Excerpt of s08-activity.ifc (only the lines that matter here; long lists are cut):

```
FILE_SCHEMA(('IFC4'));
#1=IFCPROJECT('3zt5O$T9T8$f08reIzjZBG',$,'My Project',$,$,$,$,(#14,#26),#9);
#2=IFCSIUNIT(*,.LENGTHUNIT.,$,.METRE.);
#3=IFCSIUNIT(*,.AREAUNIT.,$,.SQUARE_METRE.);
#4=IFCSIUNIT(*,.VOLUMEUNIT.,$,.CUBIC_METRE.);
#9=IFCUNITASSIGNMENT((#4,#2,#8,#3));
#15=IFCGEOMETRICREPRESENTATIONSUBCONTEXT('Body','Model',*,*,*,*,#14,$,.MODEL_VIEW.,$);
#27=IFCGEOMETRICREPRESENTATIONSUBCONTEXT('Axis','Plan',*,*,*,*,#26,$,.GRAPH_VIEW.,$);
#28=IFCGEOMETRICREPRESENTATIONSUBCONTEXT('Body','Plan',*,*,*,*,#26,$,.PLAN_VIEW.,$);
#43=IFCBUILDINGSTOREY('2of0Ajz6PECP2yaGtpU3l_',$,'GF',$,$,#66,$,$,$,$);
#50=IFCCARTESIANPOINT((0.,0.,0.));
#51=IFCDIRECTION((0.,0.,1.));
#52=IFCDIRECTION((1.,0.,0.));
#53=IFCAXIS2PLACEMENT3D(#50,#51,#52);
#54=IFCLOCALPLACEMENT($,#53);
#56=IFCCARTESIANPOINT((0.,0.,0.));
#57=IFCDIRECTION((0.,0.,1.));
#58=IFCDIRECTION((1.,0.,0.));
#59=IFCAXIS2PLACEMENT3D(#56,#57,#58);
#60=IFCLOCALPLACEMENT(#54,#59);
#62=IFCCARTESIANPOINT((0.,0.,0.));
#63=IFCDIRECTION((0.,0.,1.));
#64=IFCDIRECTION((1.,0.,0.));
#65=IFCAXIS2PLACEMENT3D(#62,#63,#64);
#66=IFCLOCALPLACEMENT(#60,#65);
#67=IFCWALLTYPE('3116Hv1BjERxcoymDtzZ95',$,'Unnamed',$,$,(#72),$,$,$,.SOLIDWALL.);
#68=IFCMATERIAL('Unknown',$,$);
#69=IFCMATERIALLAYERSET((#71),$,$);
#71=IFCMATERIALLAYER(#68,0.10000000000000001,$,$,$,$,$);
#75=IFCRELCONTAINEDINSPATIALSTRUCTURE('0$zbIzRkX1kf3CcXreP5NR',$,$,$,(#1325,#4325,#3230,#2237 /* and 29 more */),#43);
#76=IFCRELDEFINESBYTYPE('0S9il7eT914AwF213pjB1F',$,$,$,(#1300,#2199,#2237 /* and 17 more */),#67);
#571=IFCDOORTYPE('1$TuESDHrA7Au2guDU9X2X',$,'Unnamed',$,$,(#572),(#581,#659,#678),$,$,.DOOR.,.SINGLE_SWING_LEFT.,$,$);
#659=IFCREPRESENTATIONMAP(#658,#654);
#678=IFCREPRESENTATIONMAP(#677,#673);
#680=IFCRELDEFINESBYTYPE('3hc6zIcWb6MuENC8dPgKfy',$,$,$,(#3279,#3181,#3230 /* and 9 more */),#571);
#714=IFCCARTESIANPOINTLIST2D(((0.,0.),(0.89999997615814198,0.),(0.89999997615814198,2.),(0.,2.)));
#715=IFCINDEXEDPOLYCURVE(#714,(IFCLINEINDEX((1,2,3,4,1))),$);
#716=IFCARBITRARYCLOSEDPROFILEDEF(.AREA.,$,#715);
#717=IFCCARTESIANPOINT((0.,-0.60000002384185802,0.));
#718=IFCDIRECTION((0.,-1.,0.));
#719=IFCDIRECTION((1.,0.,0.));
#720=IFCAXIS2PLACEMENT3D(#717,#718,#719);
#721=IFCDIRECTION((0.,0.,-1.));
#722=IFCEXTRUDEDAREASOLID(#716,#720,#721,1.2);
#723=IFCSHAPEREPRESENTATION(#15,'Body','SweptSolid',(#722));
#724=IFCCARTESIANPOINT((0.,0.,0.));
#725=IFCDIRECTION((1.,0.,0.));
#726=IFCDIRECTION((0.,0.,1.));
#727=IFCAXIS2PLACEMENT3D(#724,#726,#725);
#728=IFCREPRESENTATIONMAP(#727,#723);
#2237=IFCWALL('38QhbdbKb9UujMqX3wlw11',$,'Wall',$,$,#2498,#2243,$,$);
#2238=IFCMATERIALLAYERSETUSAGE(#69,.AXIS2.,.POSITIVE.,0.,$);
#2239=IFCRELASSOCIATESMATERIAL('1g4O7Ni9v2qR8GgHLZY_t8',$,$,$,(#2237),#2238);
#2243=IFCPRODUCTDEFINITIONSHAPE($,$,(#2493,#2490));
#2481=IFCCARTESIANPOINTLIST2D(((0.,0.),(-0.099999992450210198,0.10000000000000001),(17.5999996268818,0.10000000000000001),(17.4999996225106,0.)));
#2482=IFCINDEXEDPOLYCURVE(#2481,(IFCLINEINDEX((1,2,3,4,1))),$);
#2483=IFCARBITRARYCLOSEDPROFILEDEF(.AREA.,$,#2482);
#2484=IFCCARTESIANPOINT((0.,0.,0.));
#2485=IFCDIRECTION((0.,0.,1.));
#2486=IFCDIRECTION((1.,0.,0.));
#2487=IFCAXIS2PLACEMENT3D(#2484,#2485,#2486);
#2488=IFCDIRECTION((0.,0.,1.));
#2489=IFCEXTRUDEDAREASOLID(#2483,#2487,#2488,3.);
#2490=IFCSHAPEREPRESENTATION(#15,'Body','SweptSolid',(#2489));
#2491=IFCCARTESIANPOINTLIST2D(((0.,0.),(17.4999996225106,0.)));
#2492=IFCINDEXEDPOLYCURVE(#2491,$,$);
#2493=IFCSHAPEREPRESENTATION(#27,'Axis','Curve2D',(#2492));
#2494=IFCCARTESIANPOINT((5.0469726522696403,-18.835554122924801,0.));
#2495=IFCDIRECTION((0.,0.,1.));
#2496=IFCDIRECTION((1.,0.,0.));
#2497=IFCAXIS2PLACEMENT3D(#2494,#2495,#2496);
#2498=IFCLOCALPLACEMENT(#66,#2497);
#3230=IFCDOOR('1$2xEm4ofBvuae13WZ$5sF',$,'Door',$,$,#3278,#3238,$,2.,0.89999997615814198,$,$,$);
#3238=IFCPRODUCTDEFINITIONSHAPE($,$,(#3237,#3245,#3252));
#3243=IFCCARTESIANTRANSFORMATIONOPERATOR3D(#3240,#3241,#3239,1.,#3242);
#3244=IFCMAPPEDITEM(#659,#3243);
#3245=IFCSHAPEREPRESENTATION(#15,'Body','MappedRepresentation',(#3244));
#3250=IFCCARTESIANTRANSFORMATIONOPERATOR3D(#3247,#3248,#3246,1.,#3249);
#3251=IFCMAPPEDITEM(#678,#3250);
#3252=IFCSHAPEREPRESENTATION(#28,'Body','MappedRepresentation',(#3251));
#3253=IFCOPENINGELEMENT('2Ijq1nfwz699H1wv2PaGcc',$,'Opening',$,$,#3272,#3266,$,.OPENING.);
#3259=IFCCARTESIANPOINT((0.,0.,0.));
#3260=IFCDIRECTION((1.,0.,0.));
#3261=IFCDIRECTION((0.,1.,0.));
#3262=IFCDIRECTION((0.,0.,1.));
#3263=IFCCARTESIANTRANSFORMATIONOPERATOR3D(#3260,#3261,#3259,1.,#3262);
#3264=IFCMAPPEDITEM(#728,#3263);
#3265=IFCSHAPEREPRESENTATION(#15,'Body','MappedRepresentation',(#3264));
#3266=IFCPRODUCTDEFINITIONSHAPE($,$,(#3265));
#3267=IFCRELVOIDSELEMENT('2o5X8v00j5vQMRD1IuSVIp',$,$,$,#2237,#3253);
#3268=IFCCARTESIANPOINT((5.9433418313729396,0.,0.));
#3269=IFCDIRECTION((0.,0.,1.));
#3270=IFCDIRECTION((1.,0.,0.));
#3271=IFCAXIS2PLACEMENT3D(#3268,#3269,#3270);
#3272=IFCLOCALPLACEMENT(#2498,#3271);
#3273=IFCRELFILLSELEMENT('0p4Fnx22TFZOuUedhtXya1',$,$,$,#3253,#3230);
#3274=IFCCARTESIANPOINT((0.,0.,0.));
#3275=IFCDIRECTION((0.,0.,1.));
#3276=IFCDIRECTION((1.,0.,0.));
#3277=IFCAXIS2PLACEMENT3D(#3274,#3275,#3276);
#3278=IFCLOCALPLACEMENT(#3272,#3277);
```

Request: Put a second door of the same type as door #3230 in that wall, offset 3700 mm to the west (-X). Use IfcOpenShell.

```python
import ifcopenshell
import ifcopenshell.api.feature
import ifcopenshell.api.geometry
import ifcopenshell.api.root
import ifcopenshell.geom
import ifcopenshell.util.element
import ifcopenshell.util.placement
import ifcopenshell.util.shape
import ifcopenshell.util.unit

model = ifcopenshell.open("s08-activity.ifc")
unit_scale = ifcopenshell.util.unit.calculate_unit_scale(model)
settings = ifcopenshell.geom.settings()


def volume(element):
    """Net volume in cubic metres, openings subtracted."""
    shape = ifcopenshell.geom.create_shape(settings, element)
    return ifcopenshell.util.shape.get_volume(shape.geometry)


door = model.by_id(3230)
opening = door.FillsVoids[0].RelatingOpeningElement
wall = opening.VoidsElements[0].RelatingBuildingElement
before = volume(wall)
shift = ifcopenshell.util.placement.get_local_placement(wall.ObjectPlacement)[:3, 0] * -3.7 / unit_scale

# copy_class copies the void relationship, type, container and properties, but no geometry.
new_opening = ifcopenshell.api.root.copy_class(model, product=opening)
new_opening.Representation = ifcopenshell.util.element.copy_deep(
    model, opening.Representation, exclude=["IfcGeometricRepresentationContext", "IfcRepresentationMap"]
)
new_door = ifcopenshell.api.root.copy_class(model, product=door)
new_door.Representation = ifcopenshell.util.element.copy_deep(
    model, door.Representation, exclude=["IfcGeometricRepresentationContext", "IfcRepresentationMap"]
)
ifcopenshell.api.feature.add_filling(model, opening=new_opening, element=new_door)

for old, new in ((opening, new_opening), (door, new_door)):
    matrix = ifcopenshell.util.placement.get_local_placement(old.ObjectPlacement)
    matrix[:3, 3] += shift
    ifcopenshell.api.geometry.edit_object_placement(model, product=new, matrix=matrix, is_si=False)

after = volume(wall)

print(f"wall volume {before:.3f} -> {after:.3f} m3")

model.write("s08-activity_v2.ifc")
```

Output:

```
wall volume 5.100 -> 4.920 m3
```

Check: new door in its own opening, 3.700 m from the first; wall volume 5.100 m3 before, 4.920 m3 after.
